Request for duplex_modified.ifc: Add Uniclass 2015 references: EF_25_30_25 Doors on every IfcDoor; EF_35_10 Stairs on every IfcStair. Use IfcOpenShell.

First a look at what the model holds.

```python
import ifcopenshell

model = ifcopenshell.open("duplex_modified.ifc")
print(model.schema)
print("classifications:", [c.Name for c in model.by_type("IfcClassification")])
for ifc_class in ("IfcDoor", "IfcRoof", "IfcStair", "IfcWall", "IfcWindow"):
    print(ifc_class, len(model.by_type(ifc_class)))
```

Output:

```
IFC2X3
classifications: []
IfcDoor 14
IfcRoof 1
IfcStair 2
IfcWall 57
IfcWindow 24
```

```python
import ifcopenshell
import ifcopenshell.api.classification

model = ifcopenshell.open("duplex_modified.ifc")

# IFC2X3 requires Source and Edition and has no link from the project to the system.
system = model.create_entity("IfcClassification", Source="NBS", Edition="2015", Name="Uniclass 2015")

codes = {
    "IfcDoor": ("EF_25_30_25", "Doors"),
    "IfcStair": ("EF_35_10", "Stairs"),
}
for ifc_class, (code, name) in codes.items():
    products = model.by_type(ifc_class)
    ifcopenshell.api.classification.add_reference(
        model, products=products, classification=system, identification=code, name=name
    )
    print(code, len(products))

model.write("duplex_modified_updated.ifc")
```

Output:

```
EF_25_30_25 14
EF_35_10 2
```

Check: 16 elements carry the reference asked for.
